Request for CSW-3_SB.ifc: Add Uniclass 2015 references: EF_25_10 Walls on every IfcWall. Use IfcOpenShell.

First a look at what the model holds.

```python
import ifcopenshell

model = ifcopenshell.open("CSW-3_SB.ifc")
print(model.schema)
print("classifications:", [c.Name for c in model.by_type("IfcClassification")])
for ifc_class in ("IfcDoor", "IfcRoof", "IfcStair", "IfcWall", "IfcWindow"):
    print(ifc_class, len(model.by_type(ifc_class)))
```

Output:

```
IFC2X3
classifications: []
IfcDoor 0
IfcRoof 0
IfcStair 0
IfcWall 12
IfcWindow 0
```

```python
import ifcopenshell
import ifcopenshell.api.classification

model = ifcopenshell.open("CSW-3_SB.ifc")

# IFC2X3 requires Source and Edition and has no link from the project to the system.
system = model.create_entity("IfcClassification", Source="NBS", Edition="2015", Name="Uniclass 2015")

codes = {
    "IfcWall": ("EF_25_10", "Walls"),
}
for ifc_class, (code, name) in codes.items():
    products = model.by_type(ifc_class)
    ifcopenshell.api.classification.add_reference(
        model, products=products, classification=system, identification=code, name=name
    )
    print(code, len(products))

model.write("CSW-3_SB_v2.ifc")
```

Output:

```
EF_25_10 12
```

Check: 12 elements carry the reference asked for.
